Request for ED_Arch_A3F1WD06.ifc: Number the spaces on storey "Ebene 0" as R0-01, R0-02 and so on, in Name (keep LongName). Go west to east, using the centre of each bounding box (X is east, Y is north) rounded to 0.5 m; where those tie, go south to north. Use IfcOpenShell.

First a look at what the model holds.

```python
import ifcopenshell
import ifcopenshell.util.element
import ifcopenshell.util.placement

model = ifcopenshell.open("ED_Arch_A3F1WD06.ifc")
print(model.schema)
storey = next(s for s in model.by_type("IfcBuildingStorey") if s.Name == "Ebene 0")
spaces = [e for e in ifcopenshell.util.element.get_decomposition(storey) if e.is_a("IfcSpace")]
for e in sorted(spaces, key=lambda e: e.id()):
    origin = ifcopenshell.util.placement.get_local_placement(e.ObjectPlacement)[:3, 3]
    print(e.id(), e.Name, e.LongName, origin.round(2) + 0.0, sep=" | ")
```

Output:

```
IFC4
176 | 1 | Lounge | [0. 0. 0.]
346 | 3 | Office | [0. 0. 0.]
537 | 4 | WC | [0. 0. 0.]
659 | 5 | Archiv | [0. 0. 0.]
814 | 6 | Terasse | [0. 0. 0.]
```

```python
import ifcopenshell
import ifcopenshell.geom
import ifcopenshell.util.element
import ifcopenshell.util.shape

model = ifcopenshell.open("ED_Arch_A3F1WD06.ifc")
settings = ifcopenshell.geom.settings()
settings.set("use-world-coords", True)


def centre(element):
    shape = ifcopenshell.geom.create_shape(settings, element)
    return ifcopenshell.util.shape.get_bbox_centroid(shape.geometry)


storey = next(s for s in model.by_type("IfcBuildingStorey") if s.Name == "Ebene 0")
spaces = [e for e in ifcopenshell.util.element.get_decomposition(storey) if e.is_a("IfcSpace")]

# Insertion points can sit at a corner or the storey origin, so sort by the geometry (in metres).
centres = {e: centre(e) for e in spaces}
spaces.sort(key=lambda e: (round(centres[e][0] / 0.5), centres[e][1]))

for i, e in enumerate(spaces, start=1):
    number = f"R0-{i:02d}"
    e.Name = number
    print(e.id(), number)

model.write("ED_Arch_A3F1WD06_rev.ifc")
```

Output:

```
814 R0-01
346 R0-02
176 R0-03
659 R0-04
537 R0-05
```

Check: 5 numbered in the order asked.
